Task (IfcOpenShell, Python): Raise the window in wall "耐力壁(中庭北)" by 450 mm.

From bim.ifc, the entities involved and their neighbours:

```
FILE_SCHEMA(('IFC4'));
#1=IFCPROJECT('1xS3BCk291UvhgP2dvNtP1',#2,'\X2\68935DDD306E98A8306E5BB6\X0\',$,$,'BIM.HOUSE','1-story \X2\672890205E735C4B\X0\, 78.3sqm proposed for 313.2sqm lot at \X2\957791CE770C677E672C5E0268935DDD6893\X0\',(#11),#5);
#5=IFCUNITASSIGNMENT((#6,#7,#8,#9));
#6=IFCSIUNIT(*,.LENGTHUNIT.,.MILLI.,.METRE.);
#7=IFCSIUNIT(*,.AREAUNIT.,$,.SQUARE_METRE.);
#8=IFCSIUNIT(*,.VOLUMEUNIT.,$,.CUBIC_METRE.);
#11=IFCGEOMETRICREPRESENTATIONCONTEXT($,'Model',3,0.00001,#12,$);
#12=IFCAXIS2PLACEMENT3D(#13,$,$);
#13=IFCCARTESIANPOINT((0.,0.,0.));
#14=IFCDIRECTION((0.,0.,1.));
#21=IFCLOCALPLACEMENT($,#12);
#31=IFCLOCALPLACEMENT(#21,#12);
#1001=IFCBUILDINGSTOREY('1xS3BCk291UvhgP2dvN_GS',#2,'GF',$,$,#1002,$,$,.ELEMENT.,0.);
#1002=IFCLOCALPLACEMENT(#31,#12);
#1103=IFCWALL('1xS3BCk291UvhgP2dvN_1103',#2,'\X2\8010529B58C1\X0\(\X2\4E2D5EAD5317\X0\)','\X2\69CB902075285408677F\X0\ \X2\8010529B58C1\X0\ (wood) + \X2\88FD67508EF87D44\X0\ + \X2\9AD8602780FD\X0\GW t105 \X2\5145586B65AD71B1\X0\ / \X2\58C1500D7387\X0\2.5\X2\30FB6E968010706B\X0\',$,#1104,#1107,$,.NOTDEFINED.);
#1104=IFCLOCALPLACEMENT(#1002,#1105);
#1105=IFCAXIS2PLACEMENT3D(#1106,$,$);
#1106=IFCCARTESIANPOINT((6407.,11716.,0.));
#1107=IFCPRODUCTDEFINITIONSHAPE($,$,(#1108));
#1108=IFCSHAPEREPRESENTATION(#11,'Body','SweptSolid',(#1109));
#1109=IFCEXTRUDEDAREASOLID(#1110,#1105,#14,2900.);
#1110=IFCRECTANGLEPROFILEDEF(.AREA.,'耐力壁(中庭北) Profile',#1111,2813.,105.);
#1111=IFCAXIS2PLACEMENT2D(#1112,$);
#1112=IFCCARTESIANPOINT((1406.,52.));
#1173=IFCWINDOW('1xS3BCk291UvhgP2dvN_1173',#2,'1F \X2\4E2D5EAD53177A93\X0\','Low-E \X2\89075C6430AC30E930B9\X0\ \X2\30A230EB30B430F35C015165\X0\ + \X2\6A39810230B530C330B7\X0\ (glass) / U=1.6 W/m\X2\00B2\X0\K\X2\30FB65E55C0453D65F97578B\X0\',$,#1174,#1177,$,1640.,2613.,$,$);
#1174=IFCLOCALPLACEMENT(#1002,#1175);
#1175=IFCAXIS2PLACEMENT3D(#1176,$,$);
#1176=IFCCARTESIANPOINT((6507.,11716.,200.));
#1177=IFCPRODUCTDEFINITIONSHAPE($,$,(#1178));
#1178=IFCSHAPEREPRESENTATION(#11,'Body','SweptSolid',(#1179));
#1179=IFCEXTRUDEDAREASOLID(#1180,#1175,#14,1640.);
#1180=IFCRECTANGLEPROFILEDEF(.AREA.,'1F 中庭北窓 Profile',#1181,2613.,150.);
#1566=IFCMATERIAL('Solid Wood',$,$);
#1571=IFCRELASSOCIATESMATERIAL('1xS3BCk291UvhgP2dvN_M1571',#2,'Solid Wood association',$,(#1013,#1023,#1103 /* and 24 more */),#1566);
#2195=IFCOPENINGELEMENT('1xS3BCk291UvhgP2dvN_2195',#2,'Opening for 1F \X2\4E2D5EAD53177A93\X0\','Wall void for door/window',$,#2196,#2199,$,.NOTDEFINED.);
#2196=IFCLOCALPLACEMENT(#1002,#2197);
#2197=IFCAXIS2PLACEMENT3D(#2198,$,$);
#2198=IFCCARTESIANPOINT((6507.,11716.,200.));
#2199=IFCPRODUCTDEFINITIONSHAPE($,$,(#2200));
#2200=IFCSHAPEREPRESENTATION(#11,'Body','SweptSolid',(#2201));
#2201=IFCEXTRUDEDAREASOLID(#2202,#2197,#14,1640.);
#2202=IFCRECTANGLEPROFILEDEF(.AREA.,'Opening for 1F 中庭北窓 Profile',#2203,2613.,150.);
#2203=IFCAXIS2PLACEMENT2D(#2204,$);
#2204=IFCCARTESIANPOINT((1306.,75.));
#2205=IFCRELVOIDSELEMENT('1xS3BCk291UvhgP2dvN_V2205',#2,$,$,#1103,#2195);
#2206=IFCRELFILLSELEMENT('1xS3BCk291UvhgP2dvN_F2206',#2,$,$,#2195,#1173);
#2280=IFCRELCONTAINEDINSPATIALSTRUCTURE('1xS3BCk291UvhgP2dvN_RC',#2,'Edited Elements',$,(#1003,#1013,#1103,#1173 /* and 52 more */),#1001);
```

```python
import numpy as np
import ifcopenshell
import ifcopenshell.api.geometry
import ifcopenshell.util.placement
import ifcopenshell.util.unit

model = ifcopenshell.open("bim.ifc")
unit_scale = ifcopenshell.util.unit.calculate_unit_scale(model)

window = model.by_guid("1xS3BCk291UvhgP2dvN_1173")
opening = window.FillsVoids[0].RelatingOpeningElement
dz = 0.45 / unit_scale

shift = np.array([0.0, 0.0, dz])
# The window is not placed relative to its opening, so move both.
for product in (opening, window):
    matrix = ifcopenshell.util.placement.get_local_placement(product.ObjectPlacement)
    matrix[:3, 3] += shift
    ifcopenshell.api.geometry.edit_object_placement(model, product=product, matrix=matrix, is_si=False)

print(f"moved by {dz * unit_scale:+.3f} m")

model.write("bim_rev.ifc")
```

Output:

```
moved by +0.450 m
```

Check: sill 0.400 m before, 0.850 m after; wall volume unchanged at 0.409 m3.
